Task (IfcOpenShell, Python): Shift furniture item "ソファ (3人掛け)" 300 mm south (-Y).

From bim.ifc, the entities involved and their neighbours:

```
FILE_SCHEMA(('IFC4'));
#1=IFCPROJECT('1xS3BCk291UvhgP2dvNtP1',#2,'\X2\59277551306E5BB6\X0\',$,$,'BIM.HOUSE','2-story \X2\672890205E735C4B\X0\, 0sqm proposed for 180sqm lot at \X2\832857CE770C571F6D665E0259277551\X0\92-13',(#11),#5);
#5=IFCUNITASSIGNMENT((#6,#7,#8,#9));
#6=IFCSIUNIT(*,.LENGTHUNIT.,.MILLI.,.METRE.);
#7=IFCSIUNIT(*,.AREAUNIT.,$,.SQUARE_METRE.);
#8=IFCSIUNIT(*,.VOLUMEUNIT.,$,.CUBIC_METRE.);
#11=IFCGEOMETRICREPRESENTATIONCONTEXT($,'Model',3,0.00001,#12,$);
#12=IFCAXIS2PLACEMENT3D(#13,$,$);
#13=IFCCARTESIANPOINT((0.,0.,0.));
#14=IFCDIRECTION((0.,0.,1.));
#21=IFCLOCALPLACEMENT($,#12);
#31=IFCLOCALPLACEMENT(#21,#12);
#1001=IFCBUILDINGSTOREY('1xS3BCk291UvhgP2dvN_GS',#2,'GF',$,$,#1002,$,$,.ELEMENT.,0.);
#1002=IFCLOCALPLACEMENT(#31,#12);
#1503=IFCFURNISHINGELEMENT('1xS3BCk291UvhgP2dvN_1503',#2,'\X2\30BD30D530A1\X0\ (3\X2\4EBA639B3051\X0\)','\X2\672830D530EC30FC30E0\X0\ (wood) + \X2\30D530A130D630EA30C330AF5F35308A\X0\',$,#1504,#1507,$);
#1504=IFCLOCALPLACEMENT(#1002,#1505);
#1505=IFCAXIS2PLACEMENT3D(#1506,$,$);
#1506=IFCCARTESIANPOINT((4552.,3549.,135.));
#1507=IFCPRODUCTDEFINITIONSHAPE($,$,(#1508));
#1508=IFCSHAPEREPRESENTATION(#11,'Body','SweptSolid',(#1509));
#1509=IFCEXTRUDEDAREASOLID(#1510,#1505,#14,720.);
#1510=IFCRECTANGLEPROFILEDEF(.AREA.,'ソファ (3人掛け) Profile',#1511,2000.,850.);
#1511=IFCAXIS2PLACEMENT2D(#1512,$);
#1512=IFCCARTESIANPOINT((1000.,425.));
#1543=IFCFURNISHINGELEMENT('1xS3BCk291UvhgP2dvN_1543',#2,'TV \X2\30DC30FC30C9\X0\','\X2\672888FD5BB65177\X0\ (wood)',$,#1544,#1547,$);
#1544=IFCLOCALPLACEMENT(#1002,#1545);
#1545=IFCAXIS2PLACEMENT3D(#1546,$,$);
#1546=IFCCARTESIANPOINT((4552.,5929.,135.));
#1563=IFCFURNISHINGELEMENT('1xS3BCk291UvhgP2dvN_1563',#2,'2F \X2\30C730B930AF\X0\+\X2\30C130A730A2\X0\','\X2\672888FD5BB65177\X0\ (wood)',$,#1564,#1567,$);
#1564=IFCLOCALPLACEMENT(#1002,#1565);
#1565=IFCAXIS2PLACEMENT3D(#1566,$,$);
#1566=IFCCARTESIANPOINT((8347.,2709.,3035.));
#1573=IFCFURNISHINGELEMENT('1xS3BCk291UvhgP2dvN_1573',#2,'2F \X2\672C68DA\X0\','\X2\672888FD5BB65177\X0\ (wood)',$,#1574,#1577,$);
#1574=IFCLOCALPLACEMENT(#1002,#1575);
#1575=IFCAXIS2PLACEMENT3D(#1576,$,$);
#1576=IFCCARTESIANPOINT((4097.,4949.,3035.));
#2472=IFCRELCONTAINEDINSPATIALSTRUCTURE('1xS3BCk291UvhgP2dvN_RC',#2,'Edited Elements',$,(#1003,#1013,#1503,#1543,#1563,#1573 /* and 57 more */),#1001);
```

```python
import ifcopenshell
import ifcopenshell.api.geometry
import ifcopenshell.util.placement

model = ifcopenshell.open("bim.ifc")

item = model.by_guid("1xS3BCk291UvhgP2dvN_1503")
matrix = ifcopenshell.util.placement.get_local_placement(item.ObjectPlacement)
matrix[1, 3] -= 300.0
ifcopenshell.api.geometry.edit_object_placement(model, product=item, matrix=matrix, is_si=False)

print(ifcopenshell.util.placement.get_local_placement(item.ObjectPlacement).round(3) + 0.0)

model.write("bim_edited.ifc")
```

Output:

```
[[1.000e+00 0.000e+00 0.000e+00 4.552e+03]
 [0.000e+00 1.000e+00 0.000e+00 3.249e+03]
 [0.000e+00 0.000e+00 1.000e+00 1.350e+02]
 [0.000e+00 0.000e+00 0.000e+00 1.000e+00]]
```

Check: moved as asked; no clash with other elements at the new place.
